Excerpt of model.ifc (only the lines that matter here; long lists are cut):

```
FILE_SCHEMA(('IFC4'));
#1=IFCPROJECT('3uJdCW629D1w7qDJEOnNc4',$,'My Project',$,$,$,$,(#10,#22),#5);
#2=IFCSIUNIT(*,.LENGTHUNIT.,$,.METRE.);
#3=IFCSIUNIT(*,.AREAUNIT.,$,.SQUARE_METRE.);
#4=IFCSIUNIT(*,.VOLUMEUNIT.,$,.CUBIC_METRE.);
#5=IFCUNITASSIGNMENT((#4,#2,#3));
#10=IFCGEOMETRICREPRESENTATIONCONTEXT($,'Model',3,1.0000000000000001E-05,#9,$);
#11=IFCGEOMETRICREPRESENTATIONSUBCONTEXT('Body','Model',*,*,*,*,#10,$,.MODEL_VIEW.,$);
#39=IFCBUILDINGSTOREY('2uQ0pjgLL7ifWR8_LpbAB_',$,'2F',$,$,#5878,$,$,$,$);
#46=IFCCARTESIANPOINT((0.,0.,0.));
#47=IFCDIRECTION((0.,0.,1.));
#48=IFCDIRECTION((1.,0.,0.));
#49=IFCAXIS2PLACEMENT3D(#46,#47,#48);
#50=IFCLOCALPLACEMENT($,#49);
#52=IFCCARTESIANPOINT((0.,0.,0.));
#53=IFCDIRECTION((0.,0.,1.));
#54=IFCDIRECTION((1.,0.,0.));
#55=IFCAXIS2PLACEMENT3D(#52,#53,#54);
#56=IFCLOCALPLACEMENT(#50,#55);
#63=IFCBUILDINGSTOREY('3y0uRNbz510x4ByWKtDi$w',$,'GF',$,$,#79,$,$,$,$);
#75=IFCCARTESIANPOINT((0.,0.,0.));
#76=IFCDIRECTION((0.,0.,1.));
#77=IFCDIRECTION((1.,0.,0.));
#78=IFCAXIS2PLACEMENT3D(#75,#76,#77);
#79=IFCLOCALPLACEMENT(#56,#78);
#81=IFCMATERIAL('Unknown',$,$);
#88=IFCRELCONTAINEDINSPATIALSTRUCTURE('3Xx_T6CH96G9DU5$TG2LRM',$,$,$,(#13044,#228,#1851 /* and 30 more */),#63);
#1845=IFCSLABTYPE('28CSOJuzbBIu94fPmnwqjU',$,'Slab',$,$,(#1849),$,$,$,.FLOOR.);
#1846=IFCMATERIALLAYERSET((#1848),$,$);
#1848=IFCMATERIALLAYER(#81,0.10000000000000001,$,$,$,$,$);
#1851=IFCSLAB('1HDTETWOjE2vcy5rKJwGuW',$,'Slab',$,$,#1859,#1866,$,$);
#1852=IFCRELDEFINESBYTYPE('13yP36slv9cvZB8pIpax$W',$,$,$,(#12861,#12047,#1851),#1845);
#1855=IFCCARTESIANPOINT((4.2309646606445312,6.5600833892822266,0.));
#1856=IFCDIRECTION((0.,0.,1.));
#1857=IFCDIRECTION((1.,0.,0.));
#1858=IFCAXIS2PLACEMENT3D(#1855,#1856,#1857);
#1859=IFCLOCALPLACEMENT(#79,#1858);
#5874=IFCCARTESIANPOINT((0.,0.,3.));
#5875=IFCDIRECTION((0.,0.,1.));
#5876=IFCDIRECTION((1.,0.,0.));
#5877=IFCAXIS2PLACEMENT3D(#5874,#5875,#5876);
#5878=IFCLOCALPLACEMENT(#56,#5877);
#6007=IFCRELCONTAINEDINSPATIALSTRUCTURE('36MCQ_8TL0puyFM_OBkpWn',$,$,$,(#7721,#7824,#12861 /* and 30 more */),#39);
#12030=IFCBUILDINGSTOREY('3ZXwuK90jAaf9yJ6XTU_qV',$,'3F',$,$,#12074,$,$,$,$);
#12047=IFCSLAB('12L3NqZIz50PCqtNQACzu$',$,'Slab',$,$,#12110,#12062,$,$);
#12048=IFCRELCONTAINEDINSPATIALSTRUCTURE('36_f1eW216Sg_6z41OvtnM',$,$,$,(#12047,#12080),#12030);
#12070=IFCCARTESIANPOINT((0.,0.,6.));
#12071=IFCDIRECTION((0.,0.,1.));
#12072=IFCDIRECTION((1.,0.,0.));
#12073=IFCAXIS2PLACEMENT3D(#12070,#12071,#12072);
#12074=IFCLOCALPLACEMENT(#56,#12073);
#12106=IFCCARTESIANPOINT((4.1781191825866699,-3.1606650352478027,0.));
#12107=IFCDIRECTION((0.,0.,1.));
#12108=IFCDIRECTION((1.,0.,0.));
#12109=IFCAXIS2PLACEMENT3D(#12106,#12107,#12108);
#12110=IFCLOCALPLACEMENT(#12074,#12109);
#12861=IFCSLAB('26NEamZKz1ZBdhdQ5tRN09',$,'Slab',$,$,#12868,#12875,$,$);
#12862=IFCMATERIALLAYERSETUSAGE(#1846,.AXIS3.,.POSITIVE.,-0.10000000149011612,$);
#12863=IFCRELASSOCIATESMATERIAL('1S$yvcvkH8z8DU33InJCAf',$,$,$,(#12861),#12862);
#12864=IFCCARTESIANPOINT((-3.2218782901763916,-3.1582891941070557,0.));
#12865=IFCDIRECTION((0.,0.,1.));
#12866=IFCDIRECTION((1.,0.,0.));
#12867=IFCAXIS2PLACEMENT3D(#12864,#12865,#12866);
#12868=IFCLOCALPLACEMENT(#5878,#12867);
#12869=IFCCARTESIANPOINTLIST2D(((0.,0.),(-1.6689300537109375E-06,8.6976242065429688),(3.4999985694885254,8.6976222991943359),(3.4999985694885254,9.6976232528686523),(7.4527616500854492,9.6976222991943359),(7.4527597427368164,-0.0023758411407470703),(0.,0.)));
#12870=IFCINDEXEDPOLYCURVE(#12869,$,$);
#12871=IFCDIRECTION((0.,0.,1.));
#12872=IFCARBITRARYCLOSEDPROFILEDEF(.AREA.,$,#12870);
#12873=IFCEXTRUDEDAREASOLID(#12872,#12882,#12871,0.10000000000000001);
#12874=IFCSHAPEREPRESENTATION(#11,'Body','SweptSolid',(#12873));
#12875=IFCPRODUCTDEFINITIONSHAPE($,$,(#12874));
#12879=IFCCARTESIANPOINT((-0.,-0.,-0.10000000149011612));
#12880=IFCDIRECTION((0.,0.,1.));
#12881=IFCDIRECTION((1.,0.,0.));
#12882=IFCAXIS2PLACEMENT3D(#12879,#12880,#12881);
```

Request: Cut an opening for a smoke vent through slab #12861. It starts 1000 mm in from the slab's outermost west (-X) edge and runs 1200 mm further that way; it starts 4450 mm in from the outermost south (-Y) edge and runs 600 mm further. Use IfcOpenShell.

```python
import numpy as np
import ifcopenshell
import ifcopenshell.api.feature
import ifcopenshell.api.geometry
import ifcopenshell.api.root
import ifcopenshell.geom
import ifcopenshell.util.placement
import ifcopenshell.util.representation
import ifcopenshell.util.shape
import ifcopenshell.util.unit

model = ifcopenshell.open("model.ifc")
unit_scale = ifcopenshell.util.unit.calculate_unit_scale(model)
settings = ifcopenshell.geom.settings()


def volume(element):
    """Net volume in cubic metres, openings subtracted."""
    shape = ifcopenshell.geom.create_shape(settings, element)
    return ifcopenshell.util.shape.get_volume(shape.geometry)


slab = model.by_id(12861)
before = volume(slab)

# Extent in the slab's own axes, in metres. The edges named are its -X and -Y sides.
slab_shape = ifcopenshell.geom.create_shape(settings, slab)
vertices = ifcopenshell.util.shape.get_vertices(slab_shape.geometry)
x_min, y_min, bottom = vertices.min(axis=0)
top = vertices[:, 2].max()

opening = ifcopenshell.api.root.create_entity(model, ifc_class="IfcOpeningElement", name="Smoke vent opening", predefined_type="OPENING")
context = ifcopenshell.util.representation.get_context(model, "Model", "Body", "MODEL_VIEW")
width, depth = 1.2, 0.6
outline = [(0.0, 0.0), (width, 0.0), (width, depth), (0.0, depth), (0.0, 0.0)]
# Overshoot both faces by 50 mm so the cut is clean.
shape = ifcopenshell.api.geometry.add_slab_representation(
    model, context=context, depth=top - bottom + 0.1, polyline=outline
)
ifcopenshell.api.geometry.assign_representation(model, product=opening, representation=shape)

matrix = ifcopenshell.util.placement.get_local_placement(slab.ObjectPlacement)
matrix[:, 3] = matrix @ np.append(np.array([x_min + 1, y_min + 4.45, bottom - 0.05]) / unit_scale, 1.0)
ifcopenshell.api.geometry.edit_object_placement(model, product=opening, matrix=matrix, is_si=False)
ifcopenshell.api.feature.add_feature(model, feature=opening, element=slab)

after = volume(slab)

print(f"slab volume {before:.3f} -> {after:.3f} m3")

model.write("model_rev.ifc")
```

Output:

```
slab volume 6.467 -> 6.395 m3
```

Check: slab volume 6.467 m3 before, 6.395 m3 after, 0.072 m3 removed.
